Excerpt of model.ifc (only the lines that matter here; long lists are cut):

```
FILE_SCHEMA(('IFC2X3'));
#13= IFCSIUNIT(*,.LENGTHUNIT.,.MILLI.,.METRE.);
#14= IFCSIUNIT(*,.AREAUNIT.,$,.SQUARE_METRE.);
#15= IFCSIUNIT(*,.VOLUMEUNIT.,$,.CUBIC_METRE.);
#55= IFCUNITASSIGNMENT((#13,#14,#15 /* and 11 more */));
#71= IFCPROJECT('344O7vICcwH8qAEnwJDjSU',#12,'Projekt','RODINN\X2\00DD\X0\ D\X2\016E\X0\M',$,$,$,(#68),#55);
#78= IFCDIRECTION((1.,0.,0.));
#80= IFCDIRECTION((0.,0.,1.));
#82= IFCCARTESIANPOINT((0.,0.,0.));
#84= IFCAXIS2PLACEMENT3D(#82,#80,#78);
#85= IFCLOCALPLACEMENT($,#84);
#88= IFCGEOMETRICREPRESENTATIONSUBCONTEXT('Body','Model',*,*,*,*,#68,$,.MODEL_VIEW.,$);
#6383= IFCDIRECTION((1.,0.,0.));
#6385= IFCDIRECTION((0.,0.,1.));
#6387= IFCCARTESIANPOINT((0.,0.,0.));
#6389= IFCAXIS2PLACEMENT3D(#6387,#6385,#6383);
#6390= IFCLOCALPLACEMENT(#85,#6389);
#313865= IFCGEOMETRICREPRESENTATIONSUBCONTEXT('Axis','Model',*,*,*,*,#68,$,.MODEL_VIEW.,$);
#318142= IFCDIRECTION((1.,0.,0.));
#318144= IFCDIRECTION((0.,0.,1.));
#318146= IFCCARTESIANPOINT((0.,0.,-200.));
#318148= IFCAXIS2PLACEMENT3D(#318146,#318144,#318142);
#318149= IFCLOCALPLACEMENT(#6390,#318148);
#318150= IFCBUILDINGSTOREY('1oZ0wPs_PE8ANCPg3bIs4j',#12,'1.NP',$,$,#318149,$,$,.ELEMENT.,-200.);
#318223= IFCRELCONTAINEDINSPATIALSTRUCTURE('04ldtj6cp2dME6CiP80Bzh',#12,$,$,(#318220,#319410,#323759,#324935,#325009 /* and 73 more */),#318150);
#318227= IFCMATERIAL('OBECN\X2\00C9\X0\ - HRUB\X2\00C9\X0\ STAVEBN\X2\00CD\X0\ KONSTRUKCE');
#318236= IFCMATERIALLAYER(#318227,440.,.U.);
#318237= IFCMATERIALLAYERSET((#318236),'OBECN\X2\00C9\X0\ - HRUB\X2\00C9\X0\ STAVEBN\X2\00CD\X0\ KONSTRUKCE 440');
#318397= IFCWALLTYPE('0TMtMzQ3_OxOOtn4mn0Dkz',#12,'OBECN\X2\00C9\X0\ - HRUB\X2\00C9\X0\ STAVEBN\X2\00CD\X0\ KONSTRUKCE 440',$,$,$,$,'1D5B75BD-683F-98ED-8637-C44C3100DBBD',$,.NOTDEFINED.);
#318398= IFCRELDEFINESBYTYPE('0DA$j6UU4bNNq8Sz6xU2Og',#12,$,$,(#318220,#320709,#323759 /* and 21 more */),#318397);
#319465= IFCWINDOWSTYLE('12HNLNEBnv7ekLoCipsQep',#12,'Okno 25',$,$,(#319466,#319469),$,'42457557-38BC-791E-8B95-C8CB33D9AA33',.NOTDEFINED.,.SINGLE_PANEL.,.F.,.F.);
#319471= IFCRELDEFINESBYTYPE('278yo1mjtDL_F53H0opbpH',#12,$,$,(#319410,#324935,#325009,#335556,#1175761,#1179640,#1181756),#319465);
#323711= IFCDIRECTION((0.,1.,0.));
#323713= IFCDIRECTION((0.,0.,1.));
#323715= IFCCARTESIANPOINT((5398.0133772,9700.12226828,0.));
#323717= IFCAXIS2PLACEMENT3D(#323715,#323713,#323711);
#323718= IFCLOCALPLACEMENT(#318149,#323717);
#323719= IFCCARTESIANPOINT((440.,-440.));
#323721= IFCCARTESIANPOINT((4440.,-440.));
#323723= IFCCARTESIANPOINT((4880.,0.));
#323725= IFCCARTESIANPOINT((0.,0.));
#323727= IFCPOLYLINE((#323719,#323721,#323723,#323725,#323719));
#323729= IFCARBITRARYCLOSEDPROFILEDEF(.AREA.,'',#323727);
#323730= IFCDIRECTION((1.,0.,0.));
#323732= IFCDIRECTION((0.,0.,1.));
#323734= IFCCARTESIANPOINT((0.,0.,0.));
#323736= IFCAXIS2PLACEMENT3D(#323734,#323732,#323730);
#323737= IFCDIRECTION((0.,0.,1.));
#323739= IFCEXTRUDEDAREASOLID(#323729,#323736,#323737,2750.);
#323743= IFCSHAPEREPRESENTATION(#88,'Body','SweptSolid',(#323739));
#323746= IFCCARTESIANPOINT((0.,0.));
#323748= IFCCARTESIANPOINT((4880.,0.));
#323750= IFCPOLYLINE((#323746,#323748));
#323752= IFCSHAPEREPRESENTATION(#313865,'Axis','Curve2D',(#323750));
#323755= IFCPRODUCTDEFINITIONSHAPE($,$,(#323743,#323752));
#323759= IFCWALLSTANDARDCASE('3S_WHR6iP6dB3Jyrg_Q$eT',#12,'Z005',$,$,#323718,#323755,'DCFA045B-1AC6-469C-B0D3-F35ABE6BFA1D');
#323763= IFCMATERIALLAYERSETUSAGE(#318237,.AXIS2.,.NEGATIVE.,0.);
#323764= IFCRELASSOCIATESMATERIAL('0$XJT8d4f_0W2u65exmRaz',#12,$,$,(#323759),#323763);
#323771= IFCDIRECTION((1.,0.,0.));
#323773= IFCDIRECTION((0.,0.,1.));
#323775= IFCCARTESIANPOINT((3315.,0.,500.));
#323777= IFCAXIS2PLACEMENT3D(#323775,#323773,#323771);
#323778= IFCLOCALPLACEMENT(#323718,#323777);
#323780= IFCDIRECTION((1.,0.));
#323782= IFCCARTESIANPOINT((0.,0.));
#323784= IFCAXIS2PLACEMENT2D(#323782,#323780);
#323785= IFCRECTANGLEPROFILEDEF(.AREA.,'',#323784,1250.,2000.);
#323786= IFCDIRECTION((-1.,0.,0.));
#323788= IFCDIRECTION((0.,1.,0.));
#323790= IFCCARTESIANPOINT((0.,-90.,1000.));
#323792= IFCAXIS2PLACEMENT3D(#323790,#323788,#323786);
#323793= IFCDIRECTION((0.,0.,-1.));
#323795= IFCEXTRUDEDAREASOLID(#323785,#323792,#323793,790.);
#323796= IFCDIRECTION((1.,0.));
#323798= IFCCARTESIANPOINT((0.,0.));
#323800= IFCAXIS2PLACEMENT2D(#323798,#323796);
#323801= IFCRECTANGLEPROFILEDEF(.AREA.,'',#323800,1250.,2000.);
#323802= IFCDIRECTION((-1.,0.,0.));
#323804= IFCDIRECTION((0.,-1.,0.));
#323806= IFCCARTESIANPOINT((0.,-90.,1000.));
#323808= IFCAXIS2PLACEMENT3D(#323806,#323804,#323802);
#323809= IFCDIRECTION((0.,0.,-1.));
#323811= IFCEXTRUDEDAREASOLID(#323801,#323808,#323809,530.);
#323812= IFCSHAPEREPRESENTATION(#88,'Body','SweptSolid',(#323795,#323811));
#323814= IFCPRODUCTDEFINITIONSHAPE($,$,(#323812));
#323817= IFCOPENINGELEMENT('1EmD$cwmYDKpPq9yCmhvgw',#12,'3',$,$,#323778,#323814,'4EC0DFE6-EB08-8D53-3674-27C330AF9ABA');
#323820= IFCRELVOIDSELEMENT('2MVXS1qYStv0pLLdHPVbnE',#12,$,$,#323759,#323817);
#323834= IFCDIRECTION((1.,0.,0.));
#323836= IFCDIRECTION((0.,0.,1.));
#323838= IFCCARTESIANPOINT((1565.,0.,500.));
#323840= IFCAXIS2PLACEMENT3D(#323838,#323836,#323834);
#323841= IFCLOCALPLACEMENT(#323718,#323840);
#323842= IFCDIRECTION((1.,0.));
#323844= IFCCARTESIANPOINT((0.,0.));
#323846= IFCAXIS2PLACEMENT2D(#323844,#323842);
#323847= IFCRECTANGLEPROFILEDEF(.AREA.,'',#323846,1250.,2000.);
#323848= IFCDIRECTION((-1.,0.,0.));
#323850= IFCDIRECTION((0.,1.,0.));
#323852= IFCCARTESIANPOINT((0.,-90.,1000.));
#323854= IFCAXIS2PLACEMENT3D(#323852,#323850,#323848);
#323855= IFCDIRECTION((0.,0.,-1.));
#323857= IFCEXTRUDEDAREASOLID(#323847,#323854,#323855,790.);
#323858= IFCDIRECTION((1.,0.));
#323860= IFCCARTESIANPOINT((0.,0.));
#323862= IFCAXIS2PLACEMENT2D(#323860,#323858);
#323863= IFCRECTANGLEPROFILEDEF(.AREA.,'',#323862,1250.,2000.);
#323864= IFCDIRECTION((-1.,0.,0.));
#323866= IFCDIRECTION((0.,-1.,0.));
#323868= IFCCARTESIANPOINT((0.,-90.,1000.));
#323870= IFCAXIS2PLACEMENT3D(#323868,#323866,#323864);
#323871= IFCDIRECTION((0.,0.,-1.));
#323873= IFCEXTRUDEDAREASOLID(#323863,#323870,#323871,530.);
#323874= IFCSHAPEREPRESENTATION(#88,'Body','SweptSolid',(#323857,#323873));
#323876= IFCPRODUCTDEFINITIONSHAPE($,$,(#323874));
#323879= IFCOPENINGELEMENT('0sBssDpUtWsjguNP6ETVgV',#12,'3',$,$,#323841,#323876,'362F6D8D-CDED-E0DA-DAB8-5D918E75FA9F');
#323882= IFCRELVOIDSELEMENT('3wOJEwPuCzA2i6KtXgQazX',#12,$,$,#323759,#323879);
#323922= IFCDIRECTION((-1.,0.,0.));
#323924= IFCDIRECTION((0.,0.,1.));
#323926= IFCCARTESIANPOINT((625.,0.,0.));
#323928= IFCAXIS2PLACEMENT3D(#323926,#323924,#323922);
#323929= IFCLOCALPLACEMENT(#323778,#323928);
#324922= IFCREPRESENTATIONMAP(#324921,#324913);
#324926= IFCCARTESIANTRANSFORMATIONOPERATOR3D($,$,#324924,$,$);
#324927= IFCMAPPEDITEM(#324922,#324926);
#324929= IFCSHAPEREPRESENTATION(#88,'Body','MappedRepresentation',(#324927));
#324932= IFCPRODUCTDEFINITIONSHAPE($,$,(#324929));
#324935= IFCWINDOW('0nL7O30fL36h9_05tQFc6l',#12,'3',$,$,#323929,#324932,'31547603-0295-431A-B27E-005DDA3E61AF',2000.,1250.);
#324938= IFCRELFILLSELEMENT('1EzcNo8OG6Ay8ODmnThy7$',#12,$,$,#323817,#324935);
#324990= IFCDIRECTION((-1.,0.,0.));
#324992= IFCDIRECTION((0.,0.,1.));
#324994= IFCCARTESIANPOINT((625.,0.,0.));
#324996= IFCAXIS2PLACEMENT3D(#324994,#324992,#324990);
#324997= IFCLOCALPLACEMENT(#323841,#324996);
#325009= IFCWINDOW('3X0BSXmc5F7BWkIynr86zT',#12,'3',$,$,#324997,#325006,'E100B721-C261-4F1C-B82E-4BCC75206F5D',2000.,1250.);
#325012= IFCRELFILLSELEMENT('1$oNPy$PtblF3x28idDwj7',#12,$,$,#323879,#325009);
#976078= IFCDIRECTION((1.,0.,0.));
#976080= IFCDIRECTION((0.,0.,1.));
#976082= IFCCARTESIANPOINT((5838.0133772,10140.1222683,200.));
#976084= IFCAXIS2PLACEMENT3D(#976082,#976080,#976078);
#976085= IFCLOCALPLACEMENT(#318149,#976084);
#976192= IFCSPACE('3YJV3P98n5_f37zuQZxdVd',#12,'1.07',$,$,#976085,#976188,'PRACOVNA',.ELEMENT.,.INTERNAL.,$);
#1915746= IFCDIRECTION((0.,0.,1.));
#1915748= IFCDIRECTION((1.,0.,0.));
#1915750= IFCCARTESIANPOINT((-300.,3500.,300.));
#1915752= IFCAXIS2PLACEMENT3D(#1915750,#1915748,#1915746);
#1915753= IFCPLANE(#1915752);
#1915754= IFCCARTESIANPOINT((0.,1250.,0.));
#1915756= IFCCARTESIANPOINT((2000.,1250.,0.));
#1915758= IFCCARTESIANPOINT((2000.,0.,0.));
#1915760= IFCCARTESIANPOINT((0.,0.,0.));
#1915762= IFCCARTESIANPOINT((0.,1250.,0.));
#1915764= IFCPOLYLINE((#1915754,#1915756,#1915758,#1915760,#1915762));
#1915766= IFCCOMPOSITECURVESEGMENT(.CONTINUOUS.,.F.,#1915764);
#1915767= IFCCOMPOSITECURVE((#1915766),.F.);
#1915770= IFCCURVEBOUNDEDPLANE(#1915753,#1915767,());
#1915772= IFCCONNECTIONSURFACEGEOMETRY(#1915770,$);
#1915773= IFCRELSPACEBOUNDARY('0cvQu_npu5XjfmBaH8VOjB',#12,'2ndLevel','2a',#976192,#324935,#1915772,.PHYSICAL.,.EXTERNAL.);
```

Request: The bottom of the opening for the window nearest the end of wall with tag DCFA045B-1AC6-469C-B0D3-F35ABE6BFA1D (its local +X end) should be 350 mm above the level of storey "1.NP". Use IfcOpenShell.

```python
import numpy as np
import ifcopenshell
import ifcopenshell.api.geometry
import ifcopenshell.geom
import ifcopenshell.util.element
import ifcopenshell.util.placement
import ifcopenshell.util.shape
import ifcopenshell.util.unit

model = ifcopenshell.open("model.ifc")
unit_scale = ifcopenshell.util.unit.calculate_unit_scale(model)

window = model.by_id(324935)
opening = window.FillsVoids[0].RelatingOpeningElement
storey = ifcopenshell.util.element.get_container(window, ifc_class="IfcBuildingStorey")
level = ifcopenshell.util.placement.get_local_placement(storey.ObjectPlacement)[2, 3]

# The opening's origin need not be at the sill, so measure its lowest point.
shape = ifcopenshell.geom.create_shape(ifcopenshell.geom.settings(), opening)
bottom = ifcopenshell.util.shape.get_shape_bottom_elevation(shape, shape.geometry) / unit_scale
dz = level + 350.0 - bottom

shift = np.array([0.0, 0.0, dz])
# The window is placed relative to its opening, so it follows when the opening moves.
matrix = ifcopenshell.util.placement.get_local_placement(opening.ObjectPlacement)
matrix[:3, 3] += shift
ifcopenshell.api.geometry.edit_object_placement(
    model, product=opening, matrix=matrix, is_si=False, should_transform_children=True
)

# Space boundary surfaces are stored in each space's coordinates; move them too.
for rel in window.ProvidesBoundaries:
    if not rel.ConnectionGeometry:
        continue
    surface = rel.ConnectionGeometry.SurfaceOnRelatingElement.BasisSurface
    space_matrix = ifcopenshell.util.placement.get_local_placement(rel.RelatingSpace.ObjectPlacement)
    point = np.array(surface.Position.Location.Coordinates) + space_matrix[:3, :3].T @ shift
    surface.Position = model.createIfcAxis2Placement3D(
        model.createIfcCartesianPoint(point.tolist()), surface.Position.Axis, surface.Position.RefDirection
    )

print(f"moved by {dz * unit_scale:+.3f} m")

model.write("model-out.ifc")
```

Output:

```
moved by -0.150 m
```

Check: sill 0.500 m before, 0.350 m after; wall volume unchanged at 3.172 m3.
